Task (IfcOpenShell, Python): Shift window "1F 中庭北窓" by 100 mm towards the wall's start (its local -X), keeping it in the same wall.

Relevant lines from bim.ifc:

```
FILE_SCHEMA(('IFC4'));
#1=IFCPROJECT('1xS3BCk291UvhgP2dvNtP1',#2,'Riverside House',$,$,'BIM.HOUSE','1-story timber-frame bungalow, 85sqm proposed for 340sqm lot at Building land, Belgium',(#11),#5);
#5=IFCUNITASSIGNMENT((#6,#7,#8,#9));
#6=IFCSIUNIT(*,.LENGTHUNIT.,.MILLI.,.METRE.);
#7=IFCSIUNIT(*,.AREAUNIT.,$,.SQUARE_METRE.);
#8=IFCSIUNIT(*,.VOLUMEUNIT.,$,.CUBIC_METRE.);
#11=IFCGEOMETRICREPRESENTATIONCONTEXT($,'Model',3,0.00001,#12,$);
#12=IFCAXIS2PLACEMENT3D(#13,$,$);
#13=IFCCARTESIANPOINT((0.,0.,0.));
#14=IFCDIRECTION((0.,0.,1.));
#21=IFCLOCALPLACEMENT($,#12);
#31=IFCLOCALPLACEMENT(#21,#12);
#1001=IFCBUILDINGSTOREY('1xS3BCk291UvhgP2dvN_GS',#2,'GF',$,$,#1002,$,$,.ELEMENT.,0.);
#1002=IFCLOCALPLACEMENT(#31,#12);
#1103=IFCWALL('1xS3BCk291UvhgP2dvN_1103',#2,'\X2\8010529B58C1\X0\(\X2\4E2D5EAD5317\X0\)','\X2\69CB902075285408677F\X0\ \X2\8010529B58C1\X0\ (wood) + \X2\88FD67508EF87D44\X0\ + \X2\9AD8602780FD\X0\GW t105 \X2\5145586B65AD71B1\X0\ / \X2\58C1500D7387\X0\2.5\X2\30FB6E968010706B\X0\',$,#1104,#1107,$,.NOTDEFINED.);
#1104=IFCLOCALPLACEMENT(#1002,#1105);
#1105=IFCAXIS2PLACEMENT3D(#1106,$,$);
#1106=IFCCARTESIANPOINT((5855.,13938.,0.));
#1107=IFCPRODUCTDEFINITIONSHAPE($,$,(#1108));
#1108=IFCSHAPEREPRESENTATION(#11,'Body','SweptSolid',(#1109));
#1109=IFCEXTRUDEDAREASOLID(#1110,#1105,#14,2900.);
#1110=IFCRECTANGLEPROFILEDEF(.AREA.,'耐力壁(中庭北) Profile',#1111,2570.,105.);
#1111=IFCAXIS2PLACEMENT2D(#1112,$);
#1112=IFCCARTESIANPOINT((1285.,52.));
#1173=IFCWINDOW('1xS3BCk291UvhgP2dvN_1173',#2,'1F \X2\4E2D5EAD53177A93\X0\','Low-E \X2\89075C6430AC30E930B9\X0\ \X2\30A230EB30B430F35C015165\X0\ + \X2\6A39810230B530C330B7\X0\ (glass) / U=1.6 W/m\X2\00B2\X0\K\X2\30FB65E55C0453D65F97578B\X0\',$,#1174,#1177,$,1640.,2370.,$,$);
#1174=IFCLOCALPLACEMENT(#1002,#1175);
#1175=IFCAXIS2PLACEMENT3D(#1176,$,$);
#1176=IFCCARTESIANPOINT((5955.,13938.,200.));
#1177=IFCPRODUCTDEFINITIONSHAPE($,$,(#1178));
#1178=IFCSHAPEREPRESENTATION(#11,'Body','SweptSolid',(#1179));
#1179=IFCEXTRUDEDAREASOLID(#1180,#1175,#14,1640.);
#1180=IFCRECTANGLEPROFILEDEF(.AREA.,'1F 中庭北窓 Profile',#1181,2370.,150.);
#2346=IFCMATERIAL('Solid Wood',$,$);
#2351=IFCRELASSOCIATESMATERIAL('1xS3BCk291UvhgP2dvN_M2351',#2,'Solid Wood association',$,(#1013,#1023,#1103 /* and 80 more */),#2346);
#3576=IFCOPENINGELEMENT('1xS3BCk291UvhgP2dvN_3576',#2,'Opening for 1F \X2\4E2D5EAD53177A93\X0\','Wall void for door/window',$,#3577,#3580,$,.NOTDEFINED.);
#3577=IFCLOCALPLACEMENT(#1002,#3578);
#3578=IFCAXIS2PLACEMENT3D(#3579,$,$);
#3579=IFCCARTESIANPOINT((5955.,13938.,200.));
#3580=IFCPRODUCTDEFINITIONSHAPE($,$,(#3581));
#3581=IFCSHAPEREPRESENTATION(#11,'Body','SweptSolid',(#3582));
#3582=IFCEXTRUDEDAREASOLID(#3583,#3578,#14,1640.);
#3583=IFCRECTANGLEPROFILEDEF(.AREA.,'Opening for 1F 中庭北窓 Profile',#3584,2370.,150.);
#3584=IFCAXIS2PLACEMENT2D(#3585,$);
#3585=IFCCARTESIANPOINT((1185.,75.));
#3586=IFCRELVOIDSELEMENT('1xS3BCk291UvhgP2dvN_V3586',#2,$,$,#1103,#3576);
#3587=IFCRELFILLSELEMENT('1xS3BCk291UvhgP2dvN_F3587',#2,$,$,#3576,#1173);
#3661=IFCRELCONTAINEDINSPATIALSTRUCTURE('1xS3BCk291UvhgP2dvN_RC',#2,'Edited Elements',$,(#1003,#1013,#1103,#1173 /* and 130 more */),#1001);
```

```python
import ifcopenshell
import ifcopenshell.api.geometry
import ifcopenshell.util.placement

model = ifcopenshell.open("bim.ifc")

window = model.by_id(1173)
opening = window.FillsVoids[0].RelatingOpeningElement
wall = opening.VoidsElements[0].RelatingBuildingElement

wall_matrix = ifcopenshell.util.placement.get_local_placement(wall.ObjectPlacement)
shift = wall_matrix[:3, 0] * -100.0
before = ifcopenshell.util.placement.get_local_placement(window.ObjectPlacement)[:3, 3].copy()

# The window is not placed relative to its opening, so move both.
for product in (opening, window):
    matrix = ifcopenshell.util.placement.get_local_placement(product.ObjectPlacement)
    matrix[:3, 3] += shift
    ifcopenshell.api.geometry.edit_object_placement(model, product=product, matrix=matrix, is_si=False)

after = ifcopenshell.util.placement.get_local_placement(window.ObjectPlacement)[:3, 3]
print("window moved by", (after - before).round(3) + 0.0)

model.write("bim_edited.ifc")
```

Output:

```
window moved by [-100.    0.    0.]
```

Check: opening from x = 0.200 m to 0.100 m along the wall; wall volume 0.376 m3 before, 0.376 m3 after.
